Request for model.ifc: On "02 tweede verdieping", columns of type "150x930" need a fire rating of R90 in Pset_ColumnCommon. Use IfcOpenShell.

First a look at what the model holds.

```python
import ifcopenshell
import ifcopenshell.util.element

model = ifcopenshell.open("model.ifc")
print(model.schema)
storey = next(s for s in model.by_type("IfcBuildingStorey") if s.Name == "02 tweede verdieping")
columns = [e for e in ifcopenshell.util.element.get_decomposition(storey) if e.is_a("IfcColumn")]
seen = {}
for e in columns:
    element_type = ifcopenshell.util.element.get_type(e)
    key = (element_type.Name if element_type != e and element_type else None, ifcopenshell.util.element.get_pset(e, "Pset_ColumnCommon", "FireRating"))
    seen[key] = seen.get(key, 0) + 1
for (name, value), count in sorted(seen.items(), key=str):
    print(count, "x", name, "|", value)
```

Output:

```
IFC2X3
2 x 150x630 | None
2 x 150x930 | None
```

```python
import ifcopenshell
import ifcopenshell.api.pset
import ifcopenshell.util.element

model = ifcopenshell.open("model.ifc")

storey = next(s for s in model.by_type("IfcBuildingStorey") if s.Name == "02 tweede verdieping")
columns = [e for e in ifcopenshell.util.element.get_decomposition(storey) if e.is_a("IfcColumn")]

count = 0
for e in columns:
    element_type = ifcopenshell.util.element.get_type(e)
    if element_type in (None, e) or element_type.Name != "150x930":
        continue
    # add_pset returns the element's existing set when there is one.
    pset = ifcopenshell.api.pset.add_pset(model, product=e, name="Pset_ColumnCommon")
    ifcopenshell.api.pset.edit_pset(model, pset=pset, properties={"FireRating": "R90"})
    count += 1

print(count, "columns updated")

model.write("model_v2.ifc")
```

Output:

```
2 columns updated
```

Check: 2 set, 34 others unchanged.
